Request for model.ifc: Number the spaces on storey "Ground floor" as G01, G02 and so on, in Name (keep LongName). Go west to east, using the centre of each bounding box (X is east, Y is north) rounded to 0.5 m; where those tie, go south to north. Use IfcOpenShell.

First a look at what the model holds.

```python
import ifcopenshell
import ifcopenshell.util.element
import ifcopenshell.util.placement

model = ifcopenshell.open("model.ifc")
print(model.schema)
storey = next(s for s in model.by_type("IfcBuildingStorey") if s.Name == "Ground floor")
spaces = [e for e in ifcopenshell.util.element.get_decomposition(storey) if e.is_a("IfcSpace")]
for e in sorted(spaces, key=lambda e: e.id()):
    origin = ifcopenshell.util.placement.get_local_placement(e.ObjectPlacement)[:3, 3]
    print(e.id(), e.Name, e.LongName, origin.round(2) + 0.0, sep=" | ")
```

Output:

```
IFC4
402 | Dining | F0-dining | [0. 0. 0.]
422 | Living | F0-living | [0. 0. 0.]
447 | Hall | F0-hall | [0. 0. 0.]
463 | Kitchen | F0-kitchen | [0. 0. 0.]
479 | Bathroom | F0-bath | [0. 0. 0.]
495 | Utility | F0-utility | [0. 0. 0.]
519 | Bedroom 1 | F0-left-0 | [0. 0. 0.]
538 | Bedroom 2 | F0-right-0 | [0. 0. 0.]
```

```python
import ifcopenshell
import ifcopenshell.geom
import ifcopenshell.util.element
import ifcopenshell.util.shape

model = ifcopenshell.open("model.ifc")
settings = ifcopenshell.geom.settings()
settings.set("use-world-coords", True)


def centre(element):
    shape = ifcopenshell.geom.create_shape(settings, element)
    return ifcopenshell.util.shape.get_bbox_centroid(shape.geometry)


storey = next(s for s in model.by_type("IfcBuildingStorey") if s.Name == "Ground floor")
spaces = [e for e in ifcopenshell.util.element.get_decomposition(storey) if e.is_a("IfcSpace")]

# Insertion points can sit at a corner or the storey origin, so sort by the geometry (in metres).
centres = {e: centre(e) for e in spaces}
spaces.sort(key=lambda e: (round(centres[e][0] / 0.5), centres[e][1]))

for i, e in enumerate(spaces, start=1):
    number = f"G{i:02d}"
    e.Name = number
    print(e.id(), number)

model.write("model_rev.ifc")
```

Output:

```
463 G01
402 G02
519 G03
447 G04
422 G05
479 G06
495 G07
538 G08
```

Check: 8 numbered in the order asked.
